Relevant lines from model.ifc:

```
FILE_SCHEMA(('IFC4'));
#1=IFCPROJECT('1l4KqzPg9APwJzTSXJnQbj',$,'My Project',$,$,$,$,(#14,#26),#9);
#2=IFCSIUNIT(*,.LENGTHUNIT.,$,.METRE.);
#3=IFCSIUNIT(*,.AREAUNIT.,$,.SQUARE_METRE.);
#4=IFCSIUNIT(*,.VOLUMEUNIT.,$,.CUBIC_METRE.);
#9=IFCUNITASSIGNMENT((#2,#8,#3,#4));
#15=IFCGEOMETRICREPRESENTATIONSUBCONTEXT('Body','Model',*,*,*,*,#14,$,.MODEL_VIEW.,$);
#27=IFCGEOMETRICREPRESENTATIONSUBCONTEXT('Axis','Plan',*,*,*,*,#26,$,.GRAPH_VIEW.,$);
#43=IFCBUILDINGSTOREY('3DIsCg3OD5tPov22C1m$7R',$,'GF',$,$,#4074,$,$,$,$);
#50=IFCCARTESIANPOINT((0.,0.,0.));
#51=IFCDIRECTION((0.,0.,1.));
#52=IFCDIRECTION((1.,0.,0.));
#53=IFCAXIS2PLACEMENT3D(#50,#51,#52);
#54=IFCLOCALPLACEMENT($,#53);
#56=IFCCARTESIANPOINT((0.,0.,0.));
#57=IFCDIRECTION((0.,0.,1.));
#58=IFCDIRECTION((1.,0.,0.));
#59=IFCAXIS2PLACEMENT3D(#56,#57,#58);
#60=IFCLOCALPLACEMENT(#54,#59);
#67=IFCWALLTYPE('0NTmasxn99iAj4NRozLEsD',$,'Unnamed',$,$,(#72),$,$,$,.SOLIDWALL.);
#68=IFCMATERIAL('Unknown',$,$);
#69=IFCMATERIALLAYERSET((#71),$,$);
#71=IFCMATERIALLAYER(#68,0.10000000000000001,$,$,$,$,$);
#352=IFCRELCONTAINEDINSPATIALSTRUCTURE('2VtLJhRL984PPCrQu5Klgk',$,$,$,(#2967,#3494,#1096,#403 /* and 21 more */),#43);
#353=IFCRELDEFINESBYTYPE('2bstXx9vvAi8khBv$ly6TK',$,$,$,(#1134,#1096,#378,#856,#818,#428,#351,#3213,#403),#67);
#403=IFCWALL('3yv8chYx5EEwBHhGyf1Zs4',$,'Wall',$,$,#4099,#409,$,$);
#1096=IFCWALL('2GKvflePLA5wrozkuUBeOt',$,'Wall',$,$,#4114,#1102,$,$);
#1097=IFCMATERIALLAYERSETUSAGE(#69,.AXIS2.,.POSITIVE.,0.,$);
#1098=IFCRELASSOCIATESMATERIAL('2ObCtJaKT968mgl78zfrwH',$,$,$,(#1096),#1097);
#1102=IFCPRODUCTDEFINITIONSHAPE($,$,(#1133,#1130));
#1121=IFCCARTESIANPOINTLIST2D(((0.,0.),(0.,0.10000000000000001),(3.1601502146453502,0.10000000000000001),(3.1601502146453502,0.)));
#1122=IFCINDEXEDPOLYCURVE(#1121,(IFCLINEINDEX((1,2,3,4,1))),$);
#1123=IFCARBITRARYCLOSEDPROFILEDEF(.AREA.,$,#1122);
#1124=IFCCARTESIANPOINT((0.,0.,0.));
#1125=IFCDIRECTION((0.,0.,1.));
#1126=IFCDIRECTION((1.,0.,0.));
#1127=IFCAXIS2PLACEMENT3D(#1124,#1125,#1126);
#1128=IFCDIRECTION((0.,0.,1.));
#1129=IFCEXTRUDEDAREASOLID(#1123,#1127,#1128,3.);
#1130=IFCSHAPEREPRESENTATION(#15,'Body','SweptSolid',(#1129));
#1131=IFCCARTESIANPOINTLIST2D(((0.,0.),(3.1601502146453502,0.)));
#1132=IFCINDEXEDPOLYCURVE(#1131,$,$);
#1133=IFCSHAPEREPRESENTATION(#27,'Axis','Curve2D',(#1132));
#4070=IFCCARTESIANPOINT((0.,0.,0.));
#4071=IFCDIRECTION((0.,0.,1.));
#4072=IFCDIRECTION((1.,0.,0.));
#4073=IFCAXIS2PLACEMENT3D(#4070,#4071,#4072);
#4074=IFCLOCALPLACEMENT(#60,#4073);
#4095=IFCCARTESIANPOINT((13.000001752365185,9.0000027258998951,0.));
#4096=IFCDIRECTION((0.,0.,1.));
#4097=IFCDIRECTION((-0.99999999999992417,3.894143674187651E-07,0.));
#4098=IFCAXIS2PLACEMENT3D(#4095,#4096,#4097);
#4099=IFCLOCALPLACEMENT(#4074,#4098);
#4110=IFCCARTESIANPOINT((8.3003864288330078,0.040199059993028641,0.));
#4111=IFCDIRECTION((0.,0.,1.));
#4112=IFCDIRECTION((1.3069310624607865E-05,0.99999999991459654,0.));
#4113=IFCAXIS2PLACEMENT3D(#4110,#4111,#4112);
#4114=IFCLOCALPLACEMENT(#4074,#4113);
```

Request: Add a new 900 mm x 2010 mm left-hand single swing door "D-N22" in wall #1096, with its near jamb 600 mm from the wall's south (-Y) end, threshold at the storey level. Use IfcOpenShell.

```python
import numpy as np
import ifcopenshell
import ifcopenshell.api.feature
import ifcopenshell.api.geometry
import ifcopenshell.api.root
import ifcopenshell.api.spatial
import ifcopenshell.geom
import ifcopenshell.util.element
import ifcopenshell.util.placement
import ifcopenshell.util.representation
import ifcopenshell.util.shape
import ifcopenshell.util.unit

model = ifcopenshell.open("model.ifc")
unit_scale = ifcopenshell.util.unit.calculate_unit_scale(model)
settings = ifcopenshell.geom.settings()


def volume(element):
    """Net volume in cubic metres, openings subtracted."""
    shape = ifcopenshell.geom.create_shape(settings, element)
    return ifcopenshell.util.shape.get_volume(shape.geometry)


wall = model.by_guid("2GKvflePLA5wrozkuUBeOt")
storey = ifcopenshell.util.element.get_container(wall, ifc_class="IfcBuildingStorey")
context = ifcopenshell.util.representation.get_context(model, "Model", "Body", "MODEL_VIEW")
before = volume(wall)

width, height, from_end, sill = 0.9, 2.01, 0.6, 0.0  # metres

# The wall runs along its own X axis, and the end named is its -X end.
wall_shape = ifcopenshell.geom.create_shape(settings, wall)
x, y, z = ifcopenshell.util.shape.get_vertices(wall_shape.geometry).T
start = x.min() + from_end
face, thickness = float(y.min()), float(y.max() - y.min())
wall_matrix = ifcopenshell.util.placement.get_local_placement(wall.ObjectPlacement)
level = ifcopenshell.util.placement.get_local_placement(storey.ObjectPlacement)[2, 3]


def in_wall(x, y):
    """Placement at x, y metres in the wall's axes, at sill height."""
    matrix = wall_matrix.copy()
    matrix[:, 3] = wall_matrix @ np.array([x / unit_scale, y / unit_scale, 0.0, 1.0])
    matrix[2, 3] = level + sill / unit_scale
    return matrix


# Opening: a box that overshoots both wall faces by 50 mm.
opening = ifcopenshell.api.root.create_entity(model, ifc_class="IfcOpeningElement", predefined_type="OPENING")
box = ifcopenshell.api.geometry.add_wall_representation(
    model, context=context, length=width, height=height, thickness=thickness + 0.1
)
ifcopenshell.api.geometry.assign_representation(model, product=opening, representation=box)
ifcopenshell.api.geometry.edit_object_placement(model, product=opening, matrix=in_wall(start, face - 0.05), is_si=False)
ifcopenshell.api.feature.add_feature(model, feature=opening, element=wall)

door = ifcopenshell.api.root.create_entity(model, ifc_class="IfcDoor", name="D-N22", predefined_type="DOOR")
door.OverallWidth, door.OverallHeight = width / unit_scale, height / unit_scale
door.OperationType = "SINGLE_SWING_LEFT"
body = ifcopenshell.api.geometry.add_door_representation(
    model,
    context=context,
    overall_width=door.OverallWidth,
    overall_height=door.OverallHeight,
    operation_type="SINGLE_SWING_LEFT",
    lining_properties={"LiningDepth": thickness / unit_scale, "ThresholdDepth": thickness / unit_scale},
)
ifcopenshell.api.geometry.assign_representation(model, product=door, representation=body)
ifcopenshell.api.spatial.assign_container(model, products=[door], relating_structure=storey)
ifcopenshell.api.feature.add_filling(model, opening=opening, element=door)

# The lining spans the wall, so the door starts at the wall face.
ifcopenshell.api.geometry.edit_object_placement(model, product=door, matrix=in_wall(start, face), is_si=False)

after = volume(wall)

print(f"wall volume {before:.3f} -> {after:.3f} m3")

model.write("model_v2.ifc")
```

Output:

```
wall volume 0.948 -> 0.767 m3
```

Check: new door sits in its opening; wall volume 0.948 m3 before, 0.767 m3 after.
